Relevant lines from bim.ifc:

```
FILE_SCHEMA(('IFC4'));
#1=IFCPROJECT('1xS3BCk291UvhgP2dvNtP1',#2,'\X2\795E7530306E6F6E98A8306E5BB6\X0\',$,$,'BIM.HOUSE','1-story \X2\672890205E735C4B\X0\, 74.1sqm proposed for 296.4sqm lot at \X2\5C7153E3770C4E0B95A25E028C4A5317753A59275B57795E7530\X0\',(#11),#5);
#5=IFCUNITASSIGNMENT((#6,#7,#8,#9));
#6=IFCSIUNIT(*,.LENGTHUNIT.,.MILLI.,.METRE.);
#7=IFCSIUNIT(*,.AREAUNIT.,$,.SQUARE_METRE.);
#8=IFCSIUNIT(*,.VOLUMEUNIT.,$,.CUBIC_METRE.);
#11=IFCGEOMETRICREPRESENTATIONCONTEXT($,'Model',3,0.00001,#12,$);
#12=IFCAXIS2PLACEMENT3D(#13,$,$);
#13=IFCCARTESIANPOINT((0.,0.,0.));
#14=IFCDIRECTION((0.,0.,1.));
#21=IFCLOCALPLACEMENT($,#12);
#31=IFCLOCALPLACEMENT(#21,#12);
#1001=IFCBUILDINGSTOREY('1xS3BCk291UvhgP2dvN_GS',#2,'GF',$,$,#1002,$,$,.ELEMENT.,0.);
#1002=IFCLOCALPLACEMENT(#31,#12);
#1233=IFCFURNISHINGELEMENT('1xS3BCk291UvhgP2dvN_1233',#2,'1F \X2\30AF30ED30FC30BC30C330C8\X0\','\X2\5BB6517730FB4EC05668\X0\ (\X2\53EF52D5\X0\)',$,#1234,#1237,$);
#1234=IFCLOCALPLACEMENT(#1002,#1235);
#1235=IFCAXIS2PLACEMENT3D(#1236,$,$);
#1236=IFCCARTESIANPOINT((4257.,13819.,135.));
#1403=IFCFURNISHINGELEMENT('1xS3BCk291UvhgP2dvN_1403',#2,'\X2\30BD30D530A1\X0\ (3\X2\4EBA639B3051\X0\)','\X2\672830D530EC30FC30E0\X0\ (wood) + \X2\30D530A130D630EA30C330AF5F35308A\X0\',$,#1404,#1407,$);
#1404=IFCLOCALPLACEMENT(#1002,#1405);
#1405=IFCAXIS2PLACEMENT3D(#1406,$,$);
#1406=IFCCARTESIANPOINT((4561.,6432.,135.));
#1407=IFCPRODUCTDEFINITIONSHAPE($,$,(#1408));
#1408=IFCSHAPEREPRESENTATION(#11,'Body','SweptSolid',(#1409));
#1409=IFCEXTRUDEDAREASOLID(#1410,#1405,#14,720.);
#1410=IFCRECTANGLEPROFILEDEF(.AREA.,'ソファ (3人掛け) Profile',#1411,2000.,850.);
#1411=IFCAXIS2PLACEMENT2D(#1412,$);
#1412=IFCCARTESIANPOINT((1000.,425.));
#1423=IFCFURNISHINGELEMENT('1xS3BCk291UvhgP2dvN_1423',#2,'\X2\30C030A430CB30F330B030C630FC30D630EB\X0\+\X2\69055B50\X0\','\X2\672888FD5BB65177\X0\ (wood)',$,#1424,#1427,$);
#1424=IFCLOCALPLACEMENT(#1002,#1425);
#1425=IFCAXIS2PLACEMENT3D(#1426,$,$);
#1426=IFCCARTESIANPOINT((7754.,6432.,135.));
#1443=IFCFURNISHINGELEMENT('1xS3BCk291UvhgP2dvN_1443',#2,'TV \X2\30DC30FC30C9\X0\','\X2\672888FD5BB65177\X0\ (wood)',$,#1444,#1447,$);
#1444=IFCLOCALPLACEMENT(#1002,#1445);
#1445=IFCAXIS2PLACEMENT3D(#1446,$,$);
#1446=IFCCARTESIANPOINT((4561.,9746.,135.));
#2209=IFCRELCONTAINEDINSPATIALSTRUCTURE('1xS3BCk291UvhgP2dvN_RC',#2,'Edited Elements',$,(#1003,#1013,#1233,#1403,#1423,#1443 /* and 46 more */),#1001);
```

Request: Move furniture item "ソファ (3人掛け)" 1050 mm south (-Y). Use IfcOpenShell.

```python
import ifcopenshell
import ifcopenshell.api.geometry
import ifcopenshell.util.placement
import ifcopenshell.util.unit

model = ifcopenshell.open("bim.ifc")
unit_scale = ifcopenshell.util.unit.calculate_unit_scale(model)

item = model.by_guid("1xS3BCk291UvhgP2dvN_1403")
matrix = ifcopenshell.util.placement.get_local_placement(item.ObjectPlacement)
matrix[1, 3] -= 1.05 / unit_scale
ifcopenshell.api.geometry.edit_object_placement(model, product=item, matrix=matrix, is_si=False)

print(ifcopenshell.util.placement.get_local_placement(item.ObjectPlacement).round(3) + 0.0)

model.write("bim_updated.ifc")
```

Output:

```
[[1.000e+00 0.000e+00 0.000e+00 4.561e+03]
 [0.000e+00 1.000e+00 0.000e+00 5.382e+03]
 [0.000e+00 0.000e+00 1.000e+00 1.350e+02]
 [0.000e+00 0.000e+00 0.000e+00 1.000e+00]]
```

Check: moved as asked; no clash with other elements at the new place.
